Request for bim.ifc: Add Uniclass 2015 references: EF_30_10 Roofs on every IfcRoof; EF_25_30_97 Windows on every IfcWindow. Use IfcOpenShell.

First a look at what the model holds.

```python
import ifcopenshell

model = ifcopenshell.open("bim.ifc")
print(model.schema)
print("classifications:", [c.Name for c in model.by_type("IfcClassification")])
for ifc_class in ("IfcDoor", "IfcRoof", "IfcStair", "IfcWall", "IfcWindow"):
    print(ifc_class, len(model.by_type(ifc_class)))
```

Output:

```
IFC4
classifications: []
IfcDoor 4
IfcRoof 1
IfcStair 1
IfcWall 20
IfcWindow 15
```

```python
import ifcopenshell
import ifcopenshell.api.classification

model = ifcopenshell.open("bim.ifc")

system = ifcopenshell.api.classification.add_classification(model, classification="Uniclass 2015")

codes = {
    "IfcRoof": ("EF_30_10", "Roofs"),
    "IfcWindow": ("EF_25_30_97", "Windows"),
}
for ifc_class, (code, name) in codes.items():
    products = model.by_type(ifc_class)
    ifcopenshell.api.classification.add_reference(
        model, products=products, classification=system, identification=code, name=name
    )
    print(code, len(products))

model.write("bim_edited.ifc")
```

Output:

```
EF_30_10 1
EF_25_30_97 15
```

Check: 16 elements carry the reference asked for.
